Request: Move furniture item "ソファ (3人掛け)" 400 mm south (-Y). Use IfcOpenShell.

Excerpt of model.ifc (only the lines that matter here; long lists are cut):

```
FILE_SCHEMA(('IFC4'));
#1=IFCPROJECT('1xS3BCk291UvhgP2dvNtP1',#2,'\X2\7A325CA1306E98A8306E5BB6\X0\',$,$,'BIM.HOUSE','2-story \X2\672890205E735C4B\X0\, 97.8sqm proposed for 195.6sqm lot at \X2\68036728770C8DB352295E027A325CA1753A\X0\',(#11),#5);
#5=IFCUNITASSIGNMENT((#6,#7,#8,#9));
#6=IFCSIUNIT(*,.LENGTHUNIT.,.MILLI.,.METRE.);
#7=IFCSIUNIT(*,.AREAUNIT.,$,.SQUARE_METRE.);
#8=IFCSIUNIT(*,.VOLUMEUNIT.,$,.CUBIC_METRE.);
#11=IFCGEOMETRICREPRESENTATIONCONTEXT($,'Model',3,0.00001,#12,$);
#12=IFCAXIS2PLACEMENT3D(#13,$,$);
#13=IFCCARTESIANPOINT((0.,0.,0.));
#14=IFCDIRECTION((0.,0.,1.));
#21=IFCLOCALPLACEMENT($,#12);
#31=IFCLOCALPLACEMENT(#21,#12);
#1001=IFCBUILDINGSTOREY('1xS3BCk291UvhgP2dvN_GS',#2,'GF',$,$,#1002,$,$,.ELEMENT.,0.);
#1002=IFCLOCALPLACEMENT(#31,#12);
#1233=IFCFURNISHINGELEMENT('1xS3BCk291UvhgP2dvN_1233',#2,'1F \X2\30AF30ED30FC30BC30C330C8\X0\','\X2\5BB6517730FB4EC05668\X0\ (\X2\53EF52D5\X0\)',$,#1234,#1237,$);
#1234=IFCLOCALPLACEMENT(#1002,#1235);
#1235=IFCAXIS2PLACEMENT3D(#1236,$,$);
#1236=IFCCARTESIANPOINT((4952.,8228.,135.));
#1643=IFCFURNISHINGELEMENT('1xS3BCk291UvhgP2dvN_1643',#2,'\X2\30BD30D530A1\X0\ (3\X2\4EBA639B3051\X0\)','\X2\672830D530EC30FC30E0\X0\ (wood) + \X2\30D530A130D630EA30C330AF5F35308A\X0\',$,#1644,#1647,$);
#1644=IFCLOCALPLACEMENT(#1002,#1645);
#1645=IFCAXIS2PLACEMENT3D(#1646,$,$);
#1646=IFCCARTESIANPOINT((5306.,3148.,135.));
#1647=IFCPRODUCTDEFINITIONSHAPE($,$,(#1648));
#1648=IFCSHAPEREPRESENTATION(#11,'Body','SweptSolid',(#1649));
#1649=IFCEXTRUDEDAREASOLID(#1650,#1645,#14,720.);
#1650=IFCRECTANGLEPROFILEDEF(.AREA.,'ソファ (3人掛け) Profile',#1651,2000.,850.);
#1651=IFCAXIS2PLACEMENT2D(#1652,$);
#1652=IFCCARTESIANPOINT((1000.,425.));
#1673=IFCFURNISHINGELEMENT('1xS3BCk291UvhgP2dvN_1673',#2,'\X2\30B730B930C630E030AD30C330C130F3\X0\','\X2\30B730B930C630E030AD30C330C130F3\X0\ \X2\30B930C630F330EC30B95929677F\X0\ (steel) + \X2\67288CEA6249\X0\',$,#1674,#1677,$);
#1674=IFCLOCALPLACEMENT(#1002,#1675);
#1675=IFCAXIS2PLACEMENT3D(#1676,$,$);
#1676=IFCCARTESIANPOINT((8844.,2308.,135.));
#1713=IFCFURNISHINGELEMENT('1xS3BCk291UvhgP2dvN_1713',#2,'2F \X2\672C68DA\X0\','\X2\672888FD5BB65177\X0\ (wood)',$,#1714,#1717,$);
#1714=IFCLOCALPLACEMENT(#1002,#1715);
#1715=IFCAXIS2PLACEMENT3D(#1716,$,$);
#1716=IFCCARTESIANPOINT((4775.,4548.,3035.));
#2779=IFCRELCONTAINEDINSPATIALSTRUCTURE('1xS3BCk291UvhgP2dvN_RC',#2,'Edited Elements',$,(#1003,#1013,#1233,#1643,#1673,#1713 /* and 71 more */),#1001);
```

```python
import ifcopenshell
import ifcopenshell.api.geometry
import ifcopenshell.util.placement
import ifcopenshell.util.unit

model = ifcopenshell.open("model.ifc")
unit_scale = ifcopenshell.util.unit.calculate_unit_scale(model)

item = model.by_id(1643)
matrix = ifcopenshell.util.placement.get_local_placement(item.ObjectPlacement)
matrix[1, 3] -= 0.4 / unit_scale
ifcopenshell.api.geometry.edit_object_placement(model, product=item, matrix=matrix, is_si=False)

print(ifcopenshell.util.placement.get_local_placement(item.ObjectPlacement).round(3) + 0.0)

model.write("model_edited.ifc")
```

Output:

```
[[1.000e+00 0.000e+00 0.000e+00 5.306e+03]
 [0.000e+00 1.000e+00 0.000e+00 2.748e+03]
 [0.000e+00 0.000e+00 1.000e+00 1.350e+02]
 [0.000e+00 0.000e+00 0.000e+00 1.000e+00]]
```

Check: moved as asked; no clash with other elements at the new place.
